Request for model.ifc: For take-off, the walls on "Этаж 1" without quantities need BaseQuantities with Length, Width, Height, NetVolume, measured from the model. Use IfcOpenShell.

First a look at what the model holds.

```python
import ifcopenshell
import ifcopenshell.util.element
import ifcopenshell.util.unit

model = ifcopenshell.open("model.ifc")
print(model.schema)
for unit_type in ("LENGTHUNIT", "AREAUNIT", "VOLUMEUNIT"):
    print(unit_type, ifcopenshell.util.unit.calculate_unit_scale(model, unit_type))
storey = next(s for s in model.by_type("IfcBuildingStorey") if s.Name == "Этаж 1")
walls = [e for e in ifcopenshell.util.element.get_decomposition(storey) if e.is_a("IfcWall")]
for e in sorted(walls, key=lambda e: e.id()):
    print(e.id(), e.is_a(), e.Name, list(ifcopenshell.util.element.get_psets(e, qtos_only=True)), sep=" | ")
```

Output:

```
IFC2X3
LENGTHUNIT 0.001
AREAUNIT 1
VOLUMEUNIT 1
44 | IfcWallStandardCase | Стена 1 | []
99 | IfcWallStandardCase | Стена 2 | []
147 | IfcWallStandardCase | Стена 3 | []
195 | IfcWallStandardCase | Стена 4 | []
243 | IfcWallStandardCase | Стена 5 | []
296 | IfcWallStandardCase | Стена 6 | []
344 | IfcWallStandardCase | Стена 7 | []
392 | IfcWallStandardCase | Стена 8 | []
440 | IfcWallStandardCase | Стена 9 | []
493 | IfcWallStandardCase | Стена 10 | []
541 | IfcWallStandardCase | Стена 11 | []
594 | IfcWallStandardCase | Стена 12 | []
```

```python
import ifcopenshell
import ifcopenshell.api.pset
import ifcopenshell.geom
import ifcopenshell.util.element
import ifcopenshell.util.shape
import ifcopenshell.util.unit

model = ifcopenshell.open("model.ifc")
unit_scale = ifcopenshell.util.unit.calculate_unit_scale(model)
volume_scale = ifcopenshell.util.unit.calculate_unit_scale(model, "VOLUMEUNIT")
settings = ifcopenshell.geom.settings()

storey = next(s for s in model.by_type("IfcBuildingStorey") if s.Name == "Этаж 1")
walls = [e for e in ifcopenshell.util.element.get_decomposition(storey) if e.is_a("IfcWall")]

for e in sorted(walls, key=lambda e: e.id()):
    if ifcopenshell.util.element.get_psets(e, qtos_only=True, should_inherit=False):
        continue
    # Geometry comes back in metres, in the element's own axes.
    shape = ifcopenshell.geom.create_shape(settings, e)
    values = {
        "Length": ifcopenshell.util.shape.get_x(shape.geometry) / unit_scale,
        "Width": ifcopenshell.util.shape.get_y(shape.geometry) / unit_scale,
        "Height": ifcopenshell.util.shape.get_z(shape.geometry) / unit_scale,
        "NetVolume": ifcopenshell.util.shape.get_volume(shape.geometry) / volume_scale,
    }
    qto = ifcopenshell.api.pset.add_qto(model, product=e, name="BaseQuantities")
    ifcopenshell.api.pset.edit_qto(model, qto=qto, properties=values)
    print(e.id(), {k: round(v, 3) for k, v in values.items()})

model.write("model_updated.ifc")
```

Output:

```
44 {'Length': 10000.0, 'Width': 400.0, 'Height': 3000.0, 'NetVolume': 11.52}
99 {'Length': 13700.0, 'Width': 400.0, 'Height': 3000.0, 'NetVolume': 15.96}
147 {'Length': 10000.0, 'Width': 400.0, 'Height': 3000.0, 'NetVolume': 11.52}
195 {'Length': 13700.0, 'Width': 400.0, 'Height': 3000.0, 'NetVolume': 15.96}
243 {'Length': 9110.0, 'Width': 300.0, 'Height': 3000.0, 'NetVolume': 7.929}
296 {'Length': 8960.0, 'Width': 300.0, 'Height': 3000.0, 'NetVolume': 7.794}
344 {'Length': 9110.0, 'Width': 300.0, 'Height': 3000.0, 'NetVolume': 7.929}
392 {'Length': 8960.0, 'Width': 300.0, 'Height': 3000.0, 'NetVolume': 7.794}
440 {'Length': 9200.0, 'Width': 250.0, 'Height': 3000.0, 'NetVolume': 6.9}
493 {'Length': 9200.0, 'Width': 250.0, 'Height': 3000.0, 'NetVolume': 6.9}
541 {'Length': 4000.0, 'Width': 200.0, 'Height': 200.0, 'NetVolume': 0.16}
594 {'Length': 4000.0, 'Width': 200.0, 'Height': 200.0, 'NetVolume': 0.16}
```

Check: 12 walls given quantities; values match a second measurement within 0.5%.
